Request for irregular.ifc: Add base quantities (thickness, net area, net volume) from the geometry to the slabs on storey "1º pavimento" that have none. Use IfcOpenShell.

First a look at what the model holds.

```python
import ifcopenshell
import ifcopenshell.util.element
import ifcopenshell.util.unit

model = ifcopenshell.open("irregular.ifc")
print(model.schema)
for unit_type in ("LENGTHUNIT", "AREAUNIT", "VOLUMEUNIT"):
    print(unit_type, ifcopenshell.util.unit.calculate_unit_scale(model, unit_type))
storey = next(s for s in model.by_type("IfcBuildingStorey") if s.Name == "1º pavimento")
slabs = [e for e in ifcopenshell.util.element.get_decomposition(storey) if e.is_a("IfcSlab")]
for e in sorted(slabs, key=lambda e: e.id()):
    print(e.id(), e.is_a(), e.Name, list(ifcopenshell.util.element.get_psets(e, qtos_only=True)), sep=" | ")
```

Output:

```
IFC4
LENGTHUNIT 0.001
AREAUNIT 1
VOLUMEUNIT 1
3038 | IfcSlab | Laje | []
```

```python
import ifcopenshell
import ifcopenshell.api.pset
import ifcopenshell.geom
import ifcopenshell.util.element
import ifcopenshell.util.shape
import ifcopenshell.util.unit

model = ifcopenshell.open("irregular.ifc")
unit_scale = ifcopenshell.util.unit.calculate_unit_scale(model)
area_scale = ifcopenshell.util.unit.calculate_unit_scale(model, "AREAUNIT")
volume_scale = ifcopenshell.util.unit.calculate_unit_scale(model, "VOLUMEUNIT")
settings = ifcopenshell.geom.settings()

storey = next(s for s in model.by_type("IfcBuildingStorey") if s.Name == "1º pavimento")
slabs = [e for e in ifcopenshell.util.element.get_decomposition(storey) if e.is_a("IfcSlab")]

for e in sorted(slabs, key=lambda e: e.id()):
    if ifcopenshell.util.element.get_psets(e, qtos_only=True, should_inherit=False):
        continue
    # Geometry comes back in metres, in the element's own axes.
    shape = ifcopenshell.geom.create_shape(settings, e)
    values = {
        "Width": ifcopenshell.util.shape.get_z(shape.geometry) / unit_scale,
        "NetArea": ifcopenshell.util.shape.get_footprint_area(shape.geometry) / area_scale,
        "NetVolume": ifcopenshell.util.shape.get_volume(shape.geometry) / volume_scale,
    }
    qto = ifcopenshell.api.pset.add_qto(model, product=e, name="Qto_SlabBaseQuantities")
    ifcopenshell.api.pset.edit_qto(model, qto=qto, properties=values)
    print(e.id(), {k: round(v, 3) for k, v in values.items()})

model.write("irregular_v2.ifc")
```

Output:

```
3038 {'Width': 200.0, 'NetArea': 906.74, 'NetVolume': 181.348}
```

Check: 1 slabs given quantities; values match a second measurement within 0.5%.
